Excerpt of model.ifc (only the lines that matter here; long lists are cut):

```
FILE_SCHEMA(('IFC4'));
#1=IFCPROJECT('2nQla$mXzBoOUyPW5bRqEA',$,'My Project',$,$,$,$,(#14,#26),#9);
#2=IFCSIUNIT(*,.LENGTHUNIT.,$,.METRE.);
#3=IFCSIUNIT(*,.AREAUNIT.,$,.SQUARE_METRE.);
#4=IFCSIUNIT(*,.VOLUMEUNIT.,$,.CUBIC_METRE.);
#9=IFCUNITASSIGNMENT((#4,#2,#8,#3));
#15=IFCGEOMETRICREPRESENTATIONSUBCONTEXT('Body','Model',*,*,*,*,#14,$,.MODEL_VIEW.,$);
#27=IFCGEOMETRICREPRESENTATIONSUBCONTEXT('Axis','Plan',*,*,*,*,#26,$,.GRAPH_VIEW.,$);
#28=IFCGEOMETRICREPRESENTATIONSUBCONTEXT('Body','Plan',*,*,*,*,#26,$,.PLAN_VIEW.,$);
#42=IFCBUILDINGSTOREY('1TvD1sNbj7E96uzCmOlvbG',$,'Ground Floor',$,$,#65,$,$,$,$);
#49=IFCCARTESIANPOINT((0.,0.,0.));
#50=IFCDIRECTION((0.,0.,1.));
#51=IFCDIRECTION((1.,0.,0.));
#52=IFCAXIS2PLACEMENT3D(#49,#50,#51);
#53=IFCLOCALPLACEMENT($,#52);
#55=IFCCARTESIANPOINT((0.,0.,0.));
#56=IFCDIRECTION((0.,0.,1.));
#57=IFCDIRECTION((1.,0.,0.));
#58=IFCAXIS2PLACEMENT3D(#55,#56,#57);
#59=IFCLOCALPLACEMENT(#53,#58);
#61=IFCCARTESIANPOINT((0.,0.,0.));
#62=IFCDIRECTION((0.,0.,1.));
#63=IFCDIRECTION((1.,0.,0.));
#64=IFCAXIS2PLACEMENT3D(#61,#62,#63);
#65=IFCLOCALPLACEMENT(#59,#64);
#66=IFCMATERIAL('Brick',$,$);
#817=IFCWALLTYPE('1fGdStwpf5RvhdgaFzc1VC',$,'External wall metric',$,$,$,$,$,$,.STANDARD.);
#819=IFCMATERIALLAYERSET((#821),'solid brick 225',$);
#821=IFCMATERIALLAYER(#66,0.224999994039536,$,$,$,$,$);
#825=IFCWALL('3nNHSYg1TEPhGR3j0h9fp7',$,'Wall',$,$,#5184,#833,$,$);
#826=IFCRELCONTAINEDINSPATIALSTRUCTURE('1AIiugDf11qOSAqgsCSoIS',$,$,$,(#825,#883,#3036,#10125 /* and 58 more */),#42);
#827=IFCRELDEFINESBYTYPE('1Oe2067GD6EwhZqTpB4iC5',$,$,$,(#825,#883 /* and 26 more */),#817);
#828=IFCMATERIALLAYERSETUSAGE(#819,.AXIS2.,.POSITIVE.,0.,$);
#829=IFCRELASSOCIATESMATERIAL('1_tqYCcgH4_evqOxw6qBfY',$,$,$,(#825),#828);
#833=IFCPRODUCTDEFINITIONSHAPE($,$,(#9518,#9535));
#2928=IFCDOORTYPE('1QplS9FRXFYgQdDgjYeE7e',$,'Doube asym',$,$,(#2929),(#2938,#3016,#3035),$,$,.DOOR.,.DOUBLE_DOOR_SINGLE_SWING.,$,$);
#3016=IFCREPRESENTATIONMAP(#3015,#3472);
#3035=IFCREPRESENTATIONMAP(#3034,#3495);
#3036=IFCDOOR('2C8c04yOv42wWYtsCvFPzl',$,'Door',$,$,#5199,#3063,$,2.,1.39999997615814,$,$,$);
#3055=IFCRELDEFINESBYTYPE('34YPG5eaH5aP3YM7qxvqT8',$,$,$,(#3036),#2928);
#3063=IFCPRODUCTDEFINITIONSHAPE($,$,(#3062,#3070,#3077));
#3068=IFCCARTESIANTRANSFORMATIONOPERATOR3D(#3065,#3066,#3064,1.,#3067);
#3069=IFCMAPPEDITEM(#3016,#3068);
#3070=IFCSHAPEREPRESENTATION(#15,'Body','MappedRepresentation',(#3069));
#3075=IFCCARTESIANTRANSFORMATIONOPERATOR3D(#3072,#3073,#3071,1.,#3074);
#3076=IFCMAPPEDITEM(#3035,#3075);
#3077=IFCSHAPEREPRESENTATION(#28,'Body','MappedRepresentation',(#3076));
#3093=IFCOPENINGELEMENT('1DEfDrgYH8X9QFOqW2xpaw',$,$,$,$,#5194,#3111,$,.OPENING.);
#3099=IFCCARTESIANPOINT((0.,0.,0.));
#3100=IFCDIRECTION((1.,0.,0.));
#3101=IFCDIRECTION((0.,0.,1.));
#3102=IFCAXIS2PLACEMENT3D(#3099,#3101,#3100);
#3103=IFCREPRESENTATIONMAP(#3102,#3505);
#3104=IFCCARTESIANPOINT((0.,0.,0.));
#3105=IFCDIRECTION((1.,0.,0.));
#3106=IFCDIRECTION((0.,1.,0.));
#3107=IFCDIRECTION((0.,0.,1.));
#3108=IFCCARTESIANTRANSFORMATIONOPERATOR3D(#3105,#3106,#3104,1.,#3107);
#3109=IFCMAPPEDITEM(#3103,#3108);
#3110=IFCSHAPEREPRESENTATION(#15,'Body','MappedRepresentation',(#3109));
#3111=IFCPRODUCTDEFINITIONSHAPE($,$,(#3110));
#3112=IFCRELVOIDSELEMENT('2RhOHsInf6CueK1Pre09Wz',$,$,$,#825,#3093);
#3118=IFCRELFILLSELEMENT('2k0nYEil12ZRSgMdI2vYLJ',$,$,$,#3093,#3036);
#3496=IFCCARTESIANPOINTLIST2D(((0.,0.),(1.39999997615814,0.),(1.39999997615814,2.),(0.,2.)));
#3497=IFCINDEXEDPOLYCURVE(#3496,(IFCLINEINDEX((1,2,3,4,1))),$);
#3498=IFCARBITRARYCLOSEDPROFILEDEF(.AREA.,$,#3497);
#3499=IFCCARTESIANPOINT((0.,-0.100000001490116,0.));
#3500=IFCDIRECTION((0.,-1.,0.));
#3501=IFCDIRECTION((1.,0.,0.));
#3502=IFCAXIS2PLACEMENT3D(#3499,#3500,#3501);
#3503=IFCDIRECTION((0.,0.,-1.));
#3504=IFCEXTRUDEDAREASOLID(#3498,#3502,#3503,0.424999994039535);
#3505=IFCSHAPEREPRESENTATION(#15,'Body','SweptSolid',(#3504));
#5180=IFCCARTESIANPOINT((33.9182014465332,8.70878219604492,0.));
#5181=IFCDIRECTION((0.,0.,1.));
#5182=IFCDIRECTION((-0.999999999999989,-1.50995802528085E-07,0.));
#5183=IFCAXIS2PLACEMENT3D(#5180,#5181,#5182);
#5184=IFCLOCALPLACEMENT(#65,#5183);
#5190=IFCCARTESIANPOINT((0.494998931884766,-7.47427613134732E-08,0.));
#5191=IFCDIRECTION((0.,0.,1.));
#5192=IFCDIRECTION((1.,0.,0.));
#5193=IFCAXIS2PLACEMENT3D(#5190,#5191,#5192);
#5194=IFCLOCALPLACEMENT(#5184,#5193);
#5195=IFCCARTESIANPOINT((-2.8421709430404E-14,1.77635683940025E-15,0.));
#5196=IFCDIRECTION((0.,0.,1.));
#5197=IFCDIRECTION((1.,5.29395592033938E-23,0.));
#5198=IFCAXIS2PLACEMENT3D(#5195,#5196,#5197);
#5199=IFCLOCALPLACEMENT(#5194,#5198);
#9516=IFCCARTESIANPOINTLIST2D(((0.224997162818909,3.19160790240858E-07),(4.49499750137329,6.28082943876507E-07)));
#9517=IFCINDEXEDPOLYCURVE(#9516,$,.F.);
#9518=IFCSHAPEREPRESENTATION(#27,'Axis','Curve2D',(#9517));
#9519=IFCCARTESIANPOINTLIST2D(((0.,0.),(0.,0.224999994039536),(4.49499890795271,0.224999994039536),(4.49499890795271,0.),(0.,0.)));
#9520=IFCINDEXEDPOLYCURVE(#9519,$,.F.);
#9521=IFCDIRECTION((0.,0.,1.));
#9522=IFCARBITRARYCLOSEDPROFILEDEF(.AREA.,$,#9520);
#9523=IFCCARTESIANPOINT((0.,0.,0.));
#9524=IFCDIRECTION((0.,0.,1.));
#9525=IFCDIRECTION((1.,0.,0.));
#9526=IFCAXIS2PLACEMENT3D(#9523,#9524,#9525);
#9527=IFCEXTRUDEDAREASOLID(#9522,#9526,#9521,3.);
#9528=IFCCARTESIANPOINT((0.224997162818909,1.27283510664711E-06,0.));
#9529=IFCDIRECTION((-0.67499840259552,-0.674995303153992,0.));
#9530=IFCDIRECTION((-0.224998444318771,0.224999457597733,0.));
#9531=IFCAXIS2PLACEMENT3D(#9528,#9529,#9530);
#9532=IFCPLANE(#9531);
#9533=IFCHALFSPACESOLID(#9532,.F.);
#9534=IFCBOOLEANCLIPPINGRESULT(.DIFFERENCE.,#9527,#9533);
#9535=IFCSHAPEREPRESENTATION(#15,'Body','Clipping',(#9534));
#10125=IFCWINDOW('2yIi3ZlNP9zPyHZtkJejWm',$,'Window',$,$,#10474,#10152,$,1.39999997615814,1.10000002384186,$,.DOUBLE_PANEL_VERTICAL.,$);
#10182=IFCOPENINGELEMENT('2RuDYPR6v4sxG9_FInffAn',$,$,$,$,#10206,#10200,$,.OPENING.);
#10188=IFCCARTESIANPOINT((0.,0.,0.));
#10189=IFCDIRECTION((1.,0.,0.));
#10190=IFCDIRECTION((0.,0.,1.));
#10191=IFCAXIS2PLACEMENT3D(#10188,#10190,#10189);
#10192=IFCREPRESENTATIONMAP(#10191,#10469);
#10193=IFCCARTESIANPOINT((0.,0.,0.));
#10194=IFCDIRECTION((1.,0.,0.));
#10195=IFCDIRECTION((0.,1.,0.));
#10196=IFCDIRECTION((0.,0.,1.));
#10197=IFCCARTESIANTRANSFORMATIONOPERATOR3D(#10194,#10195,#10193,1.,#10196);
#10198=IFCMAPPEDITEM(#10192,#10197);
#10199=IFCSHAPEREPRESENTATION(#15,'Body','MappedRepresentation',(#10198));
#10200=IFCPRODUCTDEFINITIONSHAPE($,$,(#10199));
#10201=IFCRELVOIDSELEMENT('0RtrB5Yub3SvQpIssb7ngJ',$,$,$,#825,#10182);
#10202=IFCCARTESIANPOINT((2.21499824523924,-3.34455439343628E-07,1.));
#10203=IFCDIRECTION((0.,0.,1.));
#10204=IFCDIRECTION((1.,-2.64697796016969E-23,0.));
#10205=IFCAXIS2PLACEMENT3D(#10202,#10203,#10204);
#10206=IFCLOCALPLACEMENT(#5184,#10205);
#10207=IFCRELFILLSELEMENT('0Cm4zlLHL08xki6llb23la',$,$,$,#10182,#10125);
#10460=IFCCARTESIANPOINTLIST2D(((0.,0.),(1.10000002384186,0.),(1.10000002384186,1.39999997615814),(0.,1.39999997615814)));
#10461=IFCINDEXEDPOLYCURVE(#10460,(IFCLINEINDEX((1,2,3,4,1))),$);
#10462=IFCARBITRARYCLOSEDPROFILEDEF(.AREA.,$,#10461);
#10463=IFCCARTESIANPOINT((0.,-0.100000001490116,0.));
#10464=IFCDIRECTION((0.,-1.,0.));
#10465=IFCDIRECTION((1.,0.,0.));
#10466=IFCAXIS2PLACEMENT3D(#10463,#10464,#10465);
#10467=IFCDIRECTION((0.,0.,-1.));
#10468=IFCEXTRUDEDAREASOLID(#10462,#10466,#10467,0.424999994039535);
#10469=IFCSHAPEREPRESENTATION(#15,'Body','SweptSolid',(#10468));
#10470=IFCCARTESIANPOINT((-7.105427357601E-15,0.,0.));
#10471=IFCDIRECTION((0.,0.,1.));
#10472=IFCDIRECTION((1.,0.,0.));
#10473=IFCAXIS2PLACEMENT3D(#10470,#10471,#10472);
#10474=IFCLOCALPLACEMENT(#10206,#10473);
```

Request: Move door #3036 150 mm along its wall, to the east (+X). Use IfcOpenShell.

```python
import ifcopenshell
import ifcopenshell.api.geometry
import ifcopenshell.util.placement
import ifcopenshell.util.unit

model = ifcopenshell.open("model.ifc")
unit_scale = ifcopenshell.util.unit.calculate_unit_scale(model)

door = model.by_id(3036)
opening = door.FillsVoids[0].RelatingOpeningElement
wall = opening.VoidsElements[0].RelatingBuildingElement

wall_matrix = ifcopenshell.util.placement.get_local_placement(wall.ObjectPlacement)
shift = wall_matrix[:3, 0] * -0.15 / unit_scale
before = ifcopenshell.util.placement.get_local_placement(door.ObjectPlacement)[:3, 3].copy()

# The door is placed relative to its opening, so it follows when the opening moves.
matrix = ifcopenshell.util.placement.get_local_placement(opening.ObjectPlacement)
matrix[:3, 3] += shift
ifcopenshell.api.geometry.edit_object_placement(
    model, product=opening, matrix=matrix, is_si=False, should_transform_children=True
)

after = ifcopenshell.util.placement.get_local_placement(door.ObjectPlacement)[:3, 3]
print("door moved by", (after - before).round(3) + 0.0)

model.write("model_edited.ifc")
```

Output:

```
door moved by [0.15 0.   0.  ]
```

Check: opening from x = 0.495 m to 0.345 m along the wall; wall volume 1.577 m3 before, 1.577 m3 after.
